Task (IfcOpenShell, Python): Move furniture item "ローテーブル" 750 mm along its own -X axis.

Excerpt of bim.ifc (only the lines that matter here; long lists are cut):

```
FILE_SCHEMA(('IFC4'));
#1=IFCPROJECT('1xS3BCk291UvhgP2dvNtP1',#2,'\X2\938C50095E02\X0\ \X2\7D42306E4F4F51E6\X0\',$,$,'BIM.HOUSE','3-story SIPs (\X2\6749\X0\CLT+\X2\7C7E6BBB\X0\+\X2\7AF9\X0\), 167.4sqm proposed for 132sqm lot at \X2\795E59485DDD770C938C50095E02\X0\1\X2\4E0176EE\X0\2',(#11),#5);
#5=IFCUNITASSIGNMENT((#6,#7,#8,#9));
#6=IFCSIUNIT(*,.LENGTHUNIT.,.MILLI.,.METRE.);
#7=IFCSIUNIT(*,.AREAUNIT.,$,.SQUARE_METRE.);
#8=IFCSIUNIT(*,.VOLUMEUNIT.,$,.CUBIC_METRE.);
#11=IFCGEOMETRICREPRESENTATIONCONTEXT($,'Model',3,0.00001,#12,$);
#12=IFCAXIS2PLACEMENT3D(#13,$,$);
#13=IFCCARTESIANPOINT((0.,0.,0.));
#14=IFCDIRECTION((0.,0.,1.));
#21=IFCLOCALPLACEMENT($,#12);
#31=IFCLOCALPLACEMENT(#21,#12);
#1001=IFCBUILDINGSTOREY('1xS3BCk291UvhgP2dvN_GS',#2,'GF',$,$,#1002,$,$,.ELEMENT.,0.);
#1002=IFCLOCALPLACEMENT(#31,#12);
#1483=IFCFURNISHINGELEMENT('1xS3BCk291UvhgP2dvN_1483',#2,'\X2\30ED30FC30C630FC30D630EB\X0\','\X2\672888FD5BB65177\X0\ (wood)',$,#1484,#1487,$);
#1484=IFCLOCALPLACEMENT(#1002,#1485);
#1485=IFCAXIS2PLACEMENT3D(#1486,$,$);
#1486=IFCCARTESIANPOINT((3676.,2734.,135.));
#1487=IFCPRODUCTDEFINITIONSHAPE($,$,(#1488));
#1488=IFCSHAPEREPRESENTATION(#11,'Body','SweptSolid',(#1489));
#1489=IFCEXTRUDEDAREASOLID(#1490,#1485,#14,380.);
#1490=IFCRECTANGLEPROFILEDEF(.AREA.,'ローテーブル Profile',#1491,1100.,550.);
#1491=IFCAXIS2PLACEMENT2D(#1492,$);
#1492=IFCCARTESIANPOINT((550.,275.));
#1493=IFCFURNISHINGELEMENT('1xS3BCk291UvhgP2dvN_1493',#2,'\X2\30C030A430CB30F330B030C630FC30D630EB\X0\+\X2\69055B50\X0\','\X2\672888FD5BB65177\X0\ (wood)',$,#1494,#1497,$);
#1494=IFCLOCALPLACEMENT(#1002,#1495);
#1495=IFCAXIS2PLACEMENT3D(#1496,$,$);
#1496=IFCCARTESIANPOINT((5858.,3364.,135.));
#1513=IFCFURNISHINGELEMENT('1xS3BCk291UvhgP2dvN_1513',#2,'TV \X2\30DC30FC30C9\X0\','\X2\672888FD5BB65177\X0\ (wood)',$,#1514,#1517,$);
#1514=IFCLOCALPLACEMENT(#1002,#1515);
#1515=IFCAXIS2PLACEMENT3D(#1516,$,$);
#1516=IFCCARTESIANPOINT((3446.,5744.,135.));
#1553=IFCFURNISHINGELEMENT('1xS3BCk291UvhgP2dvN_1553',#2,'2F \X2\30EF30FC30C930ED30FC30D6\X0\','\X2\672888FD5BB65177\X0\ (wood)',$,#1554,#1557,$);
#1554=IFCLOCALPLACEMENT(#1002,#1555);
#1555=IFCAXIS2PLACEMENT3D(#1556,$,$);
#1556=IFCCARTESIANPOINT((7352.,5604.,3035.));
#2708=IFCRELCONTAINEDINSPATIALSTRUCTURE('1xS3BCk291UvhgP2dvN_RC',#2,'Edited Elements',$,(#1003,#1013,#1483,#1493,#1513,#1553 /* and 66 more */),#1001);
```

```python
import ifcopenshell
import ifcopenshell.api.geometry
import ifcopenshell.util.placement
import ifcopenshell.util.unit

model = ifcopenshell.open("bim.ifc")
unit_scale = ifcopenshell.util.unit.calculate_unit_scale(model)

item = model.by_guid("1xS3BCk291UvhgP2dvN_1483")
matrix = ifcopenshell.util.placement.get_local_placement(item.ObjectPlacement)
matrix[:3, 3] -= matrix[:3, 0] * 0.75 / unit_scale
ifcopenshell.api.geometry.edit_object_placement(model, product=item, matrix=matrix, is_si=False)

print(ifcopenshell.util.placement.get_local_placement(item.ObjectPlacement).round(3) + 0.0)

model.write("bim_v2.ifc")
```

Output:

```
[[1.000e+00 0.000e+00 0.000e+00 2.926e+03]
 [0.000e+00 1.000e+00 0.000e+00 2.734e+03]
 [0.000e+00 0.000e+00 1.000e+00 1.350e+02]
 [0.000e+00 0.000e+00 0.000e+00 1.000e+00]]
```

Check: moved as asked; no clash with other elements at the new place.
